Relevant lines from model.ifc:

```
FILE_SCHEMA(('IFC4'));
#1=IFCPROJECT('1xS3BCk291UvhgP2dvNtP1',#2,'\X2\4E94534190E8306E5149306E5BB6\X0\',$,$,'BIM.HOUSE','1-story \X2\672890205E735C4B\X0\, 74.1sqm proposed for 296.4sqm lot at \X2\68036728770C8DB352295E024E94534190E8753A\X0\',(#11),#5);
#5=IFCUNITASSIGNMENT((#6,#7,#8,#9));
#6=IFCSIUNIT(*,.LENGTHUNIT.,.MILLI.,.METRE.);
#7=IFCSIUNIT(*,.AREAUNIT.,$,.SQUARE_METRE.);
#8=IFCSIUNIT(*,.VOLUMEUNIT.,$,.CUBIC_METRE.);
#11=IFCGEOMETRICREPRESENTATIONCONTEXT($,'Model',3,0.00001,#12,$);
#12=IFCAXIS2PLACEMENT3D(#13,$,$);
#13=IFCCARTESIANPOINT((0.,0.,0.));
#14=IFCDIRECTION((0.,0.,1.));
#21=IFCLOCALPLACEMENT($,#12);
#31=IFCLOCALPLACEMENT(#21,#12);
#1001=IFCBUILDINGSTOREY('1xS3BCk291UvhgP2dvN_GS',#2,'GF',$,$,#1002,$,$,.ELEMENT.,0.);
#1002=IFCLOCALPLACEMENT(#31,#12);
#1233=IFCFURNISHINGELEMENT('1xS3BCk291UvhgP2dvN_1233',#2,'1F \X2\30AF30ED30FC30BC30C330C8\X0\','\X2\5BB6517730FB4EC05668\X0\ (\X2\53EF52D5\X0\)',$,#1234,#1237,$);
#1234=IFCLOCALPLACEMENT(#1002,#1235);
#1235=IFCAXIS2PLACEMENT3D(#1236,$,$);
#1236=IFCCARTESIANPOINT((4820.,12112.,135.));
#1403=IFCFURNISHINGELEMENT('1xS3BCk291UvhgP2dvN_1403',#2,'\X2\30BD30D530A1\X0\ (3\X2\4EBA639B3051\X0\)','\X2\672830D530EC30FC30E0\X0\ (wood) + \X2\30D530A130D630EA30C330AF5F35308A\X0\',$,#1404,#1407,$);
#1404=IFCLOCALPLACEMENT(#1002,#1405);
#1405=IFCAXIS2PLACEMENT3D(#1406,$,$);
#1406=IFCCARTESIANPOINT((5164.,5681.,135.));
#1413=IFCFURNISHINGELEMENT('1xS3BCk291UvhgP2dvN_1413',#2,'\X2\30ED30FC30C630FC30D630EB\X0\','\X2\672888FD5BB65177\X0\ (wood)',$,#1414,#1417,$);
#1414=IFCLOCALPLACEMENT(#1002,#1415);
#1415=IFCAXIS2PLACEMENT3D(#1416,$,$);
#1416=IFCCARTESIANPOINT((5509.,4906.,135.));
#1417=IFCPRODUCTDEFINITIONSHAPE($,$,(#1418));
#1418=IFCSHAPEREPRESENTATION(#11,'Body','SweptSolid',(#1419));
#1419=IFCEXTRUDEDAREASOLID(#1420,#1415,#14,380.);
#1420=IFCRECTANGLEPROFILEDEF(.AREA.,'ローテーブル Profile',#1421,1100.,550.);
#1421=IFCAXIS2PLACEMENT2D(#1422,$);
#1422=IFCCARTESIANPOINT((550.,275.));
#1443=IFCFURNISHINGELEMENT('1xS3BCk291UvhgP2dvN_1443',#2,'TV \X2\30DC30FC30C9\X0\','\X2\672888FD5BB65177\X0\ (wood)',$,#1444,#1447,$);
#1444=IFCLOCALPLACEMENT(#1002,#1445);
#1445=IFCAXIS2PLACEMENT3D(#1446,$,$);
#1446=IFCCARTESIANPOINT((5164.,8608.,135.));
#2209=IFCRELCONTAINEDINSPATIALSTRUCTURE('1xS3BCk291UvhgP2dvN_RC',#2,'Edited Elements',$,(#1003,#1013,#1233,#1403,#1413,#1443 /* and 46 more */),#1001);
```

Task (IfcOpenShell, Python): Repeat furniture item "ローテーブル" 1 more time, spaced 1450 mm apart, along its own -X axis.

```python
import ifcopenshell
import ifcopenshell.api.geometry
import ifcopenshell.api.root
import ifcopenshell.util.element
import ifcopenshell.util.placement

model = ifcopenshell.open("model.ifc")


def reuse_history(source, copy):
    """copy_class also copies each property set's owner history, people and application; keep the originals."""
    for rel in copy.IsDefinedBy:
        if rel.is_a("IfcRelDefinesByProperties") and (history := rel.RelatingPropertyDefinition.OwnerHistory):
            rel.RelatingPropertyDefinition.OwnerHistory = source.OwnerHistory
            ifcopenshell.util.element.remove_deep2(model, history)


source = model.by_guid("1xS3BCk291UvhgP2dvN_1413")
base = ifcopenshell.util.placement.get_local_placement(source.ObjectPlacement)
step = -base[:3, 0] * 1450.0

for i in range(1, 2):
    copy = ifcopenshell.api.root.copy_class(model, product=source)
    copy.Representation = ifcopenshell.util.element.copy_deep(
        model, source.Representation, exclude=["IfcGeometricRepresentationContext", "IfcRepresentationMap"]
    )
    reuse_history(source, copy)
    matrix = base.copy()
    matrix[:3, 3] += i * step
    print("added at", matrix[:3, 3].round(3) + 0.0)
    ifcopenshell.api.geometry.edit_object_placement(model, product=copy, matrix=matrix, is_si=False)

model.write("model_edited.ifc")
```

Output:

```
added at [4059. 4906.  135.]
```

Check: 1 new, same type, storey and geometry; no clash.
